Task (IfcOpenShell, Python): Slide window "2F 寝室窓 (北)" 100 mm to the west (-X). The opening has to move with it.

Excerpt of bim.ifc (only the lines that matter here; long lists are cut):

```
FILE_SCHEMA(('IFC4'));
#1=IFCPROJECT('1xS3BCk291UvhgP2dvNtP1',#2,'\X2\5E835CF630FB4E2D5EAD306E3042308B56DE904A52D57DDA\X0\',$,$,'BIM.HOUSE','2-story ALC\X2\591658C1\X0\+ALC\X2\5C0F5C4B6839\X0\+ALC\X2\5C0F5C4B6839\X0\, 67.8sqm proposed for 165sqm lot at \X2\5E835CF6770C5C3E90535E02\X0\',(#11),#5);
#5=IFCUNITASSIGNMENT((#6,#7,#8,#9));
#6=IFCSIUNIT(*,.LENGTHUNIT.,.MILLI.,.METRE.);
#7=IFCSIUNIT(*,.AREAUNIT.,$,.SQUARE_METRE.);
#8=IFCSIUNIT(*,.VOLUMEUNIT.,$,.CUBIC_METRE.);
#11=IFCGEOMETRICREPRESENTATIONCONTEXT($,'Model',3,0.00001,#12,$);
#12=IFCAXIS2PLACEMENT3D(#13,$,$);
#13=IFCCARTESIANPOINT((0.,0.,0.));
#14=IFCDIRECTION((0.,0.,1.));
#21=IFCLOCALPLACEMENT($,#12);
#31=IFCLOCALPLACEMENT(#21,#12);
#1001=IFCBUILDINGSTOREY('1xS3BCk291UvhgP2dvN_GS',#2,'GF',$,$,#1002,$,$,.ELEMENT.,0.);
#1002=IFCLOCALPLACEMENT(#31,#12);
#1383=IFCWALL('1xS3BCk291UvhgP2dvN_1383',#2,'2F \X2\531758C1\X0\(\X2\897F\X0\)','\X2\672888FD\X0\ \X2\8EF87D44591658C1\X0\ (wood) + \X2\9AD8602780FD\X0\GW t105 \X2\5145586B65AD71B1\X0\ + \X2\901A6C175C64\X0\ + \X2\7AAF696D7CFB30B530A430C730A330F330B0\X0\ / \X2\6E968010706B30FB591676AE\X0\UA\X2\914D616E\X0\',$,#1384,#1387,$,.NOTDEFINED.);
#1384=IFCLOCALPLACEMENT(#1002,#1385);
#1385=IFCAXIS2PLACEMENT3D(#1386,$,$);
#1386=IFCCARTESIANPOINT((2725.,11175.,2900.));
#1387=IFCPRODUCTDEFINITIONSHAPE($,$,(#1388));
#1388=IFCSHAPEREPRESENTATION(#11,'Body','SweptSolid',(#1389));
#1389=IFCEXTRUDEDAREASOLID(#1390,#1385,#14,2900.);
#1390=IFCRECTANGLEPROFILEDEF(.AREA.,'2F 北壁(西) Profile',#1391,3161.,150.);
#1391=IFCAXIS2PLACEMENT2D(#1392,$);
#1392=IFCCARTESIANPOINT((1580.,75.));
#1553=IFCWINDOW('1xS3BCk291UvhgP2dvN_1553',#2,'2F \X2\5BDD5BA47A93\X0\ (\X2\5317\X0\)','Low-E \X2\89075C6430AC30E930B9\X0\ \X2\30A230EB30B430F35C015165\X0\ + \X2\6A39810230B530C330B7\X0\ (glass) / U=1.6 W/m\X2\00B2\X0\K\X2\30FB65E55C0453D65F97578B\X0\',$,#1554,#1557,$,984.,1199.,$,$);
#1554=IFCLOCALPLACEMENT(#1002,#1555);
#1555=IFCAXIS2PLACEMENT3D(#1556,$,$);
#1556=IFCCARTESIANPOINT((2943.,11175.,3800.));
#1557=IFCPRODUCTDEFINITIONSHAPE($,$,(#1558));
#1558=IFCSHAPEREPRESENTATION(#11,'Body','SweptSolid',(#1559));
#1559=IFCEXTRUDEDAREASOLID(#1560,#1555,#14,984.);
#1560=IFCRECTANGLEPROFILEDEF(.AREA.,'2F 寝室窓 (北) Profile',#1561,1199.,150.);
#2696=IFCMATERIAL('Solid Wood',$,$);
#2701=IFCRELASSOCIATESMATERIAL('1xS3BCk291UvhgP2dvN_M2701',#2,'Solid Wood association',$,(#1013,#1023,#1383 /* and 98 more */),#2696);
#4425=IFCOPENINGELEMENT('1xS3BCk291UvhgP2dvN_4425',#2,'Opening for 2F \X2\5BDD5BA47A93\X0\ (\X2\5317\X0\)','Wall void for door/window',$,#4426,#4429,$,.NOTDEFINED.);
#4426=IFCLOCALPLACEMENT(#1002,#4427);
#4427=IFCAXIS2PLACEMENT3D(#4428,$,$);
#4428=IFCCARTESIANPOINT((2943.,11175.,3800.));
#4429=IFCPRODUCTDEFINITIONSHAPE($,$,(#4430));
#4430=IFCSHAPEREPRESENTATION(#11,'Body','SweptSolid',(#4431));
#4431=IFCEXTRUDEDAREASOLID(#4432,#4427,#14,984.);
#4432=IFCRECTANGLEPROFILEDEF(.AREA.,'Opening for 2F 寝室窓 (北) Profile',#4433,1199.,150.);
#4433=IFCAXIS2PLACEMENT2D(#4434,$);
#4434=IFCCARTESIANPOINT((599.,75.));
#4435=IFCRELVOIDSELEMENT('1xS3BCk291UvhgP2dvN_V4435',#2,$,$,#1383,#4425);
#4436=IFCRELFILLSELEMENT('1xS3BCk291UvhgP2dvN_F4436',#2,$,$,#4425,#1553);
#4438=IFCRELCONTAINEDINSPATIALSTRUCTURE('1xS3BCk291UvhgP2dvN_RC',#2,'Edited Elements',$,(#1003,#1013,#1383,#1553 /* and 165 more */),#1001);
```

```python
import ifcopenshell
import ifcopenshell.api.geometry
import ifcopenshell.util.placement
import ifcopenshell.util.unit

model = ifcopenshell.open("bim.ifc")
unit_scale = ifcopenshell.util.unit.calculate_unit_scale(model)

window = model.by_id(1553)
opening = window.FillsVoids[0].RelatingOpeningElement
wall = opening.VoidsElements[0].RelatingBuildingElement

wall_matrix = ifcopenshell.util.placement.get_local_placement(wall.ObjectPlacement)
shift = wall_matrix[:3, 0] * -0.1 / unit_scale
before = ifcopenshell.util.placement.get_local_placement(window.ObjectPlacement)[:3, 3].copy()

# The window is not placed relative to its opening, so move both.
for product in (opening, window):
    matrix = ifcopenshell.util.placement.get_local_placement(product.ObjectPlacement)
    matrix[:3, 3] += shift
    ifcopenshell.api.geometry.edit_object_placement(model, product=product, matrix=matrix, is_si=False)

after = ifcopenshell.util.placement.get_local_placement(window.ObjectPlacement)[:3, 3]
print("window moved by", (after - before).round(3) + 0.0)

model.write("bim_updated.ifc")
```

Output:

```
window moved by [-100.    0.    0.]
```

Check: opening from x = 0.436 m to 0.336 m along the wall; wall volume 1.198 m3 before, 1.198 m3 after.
